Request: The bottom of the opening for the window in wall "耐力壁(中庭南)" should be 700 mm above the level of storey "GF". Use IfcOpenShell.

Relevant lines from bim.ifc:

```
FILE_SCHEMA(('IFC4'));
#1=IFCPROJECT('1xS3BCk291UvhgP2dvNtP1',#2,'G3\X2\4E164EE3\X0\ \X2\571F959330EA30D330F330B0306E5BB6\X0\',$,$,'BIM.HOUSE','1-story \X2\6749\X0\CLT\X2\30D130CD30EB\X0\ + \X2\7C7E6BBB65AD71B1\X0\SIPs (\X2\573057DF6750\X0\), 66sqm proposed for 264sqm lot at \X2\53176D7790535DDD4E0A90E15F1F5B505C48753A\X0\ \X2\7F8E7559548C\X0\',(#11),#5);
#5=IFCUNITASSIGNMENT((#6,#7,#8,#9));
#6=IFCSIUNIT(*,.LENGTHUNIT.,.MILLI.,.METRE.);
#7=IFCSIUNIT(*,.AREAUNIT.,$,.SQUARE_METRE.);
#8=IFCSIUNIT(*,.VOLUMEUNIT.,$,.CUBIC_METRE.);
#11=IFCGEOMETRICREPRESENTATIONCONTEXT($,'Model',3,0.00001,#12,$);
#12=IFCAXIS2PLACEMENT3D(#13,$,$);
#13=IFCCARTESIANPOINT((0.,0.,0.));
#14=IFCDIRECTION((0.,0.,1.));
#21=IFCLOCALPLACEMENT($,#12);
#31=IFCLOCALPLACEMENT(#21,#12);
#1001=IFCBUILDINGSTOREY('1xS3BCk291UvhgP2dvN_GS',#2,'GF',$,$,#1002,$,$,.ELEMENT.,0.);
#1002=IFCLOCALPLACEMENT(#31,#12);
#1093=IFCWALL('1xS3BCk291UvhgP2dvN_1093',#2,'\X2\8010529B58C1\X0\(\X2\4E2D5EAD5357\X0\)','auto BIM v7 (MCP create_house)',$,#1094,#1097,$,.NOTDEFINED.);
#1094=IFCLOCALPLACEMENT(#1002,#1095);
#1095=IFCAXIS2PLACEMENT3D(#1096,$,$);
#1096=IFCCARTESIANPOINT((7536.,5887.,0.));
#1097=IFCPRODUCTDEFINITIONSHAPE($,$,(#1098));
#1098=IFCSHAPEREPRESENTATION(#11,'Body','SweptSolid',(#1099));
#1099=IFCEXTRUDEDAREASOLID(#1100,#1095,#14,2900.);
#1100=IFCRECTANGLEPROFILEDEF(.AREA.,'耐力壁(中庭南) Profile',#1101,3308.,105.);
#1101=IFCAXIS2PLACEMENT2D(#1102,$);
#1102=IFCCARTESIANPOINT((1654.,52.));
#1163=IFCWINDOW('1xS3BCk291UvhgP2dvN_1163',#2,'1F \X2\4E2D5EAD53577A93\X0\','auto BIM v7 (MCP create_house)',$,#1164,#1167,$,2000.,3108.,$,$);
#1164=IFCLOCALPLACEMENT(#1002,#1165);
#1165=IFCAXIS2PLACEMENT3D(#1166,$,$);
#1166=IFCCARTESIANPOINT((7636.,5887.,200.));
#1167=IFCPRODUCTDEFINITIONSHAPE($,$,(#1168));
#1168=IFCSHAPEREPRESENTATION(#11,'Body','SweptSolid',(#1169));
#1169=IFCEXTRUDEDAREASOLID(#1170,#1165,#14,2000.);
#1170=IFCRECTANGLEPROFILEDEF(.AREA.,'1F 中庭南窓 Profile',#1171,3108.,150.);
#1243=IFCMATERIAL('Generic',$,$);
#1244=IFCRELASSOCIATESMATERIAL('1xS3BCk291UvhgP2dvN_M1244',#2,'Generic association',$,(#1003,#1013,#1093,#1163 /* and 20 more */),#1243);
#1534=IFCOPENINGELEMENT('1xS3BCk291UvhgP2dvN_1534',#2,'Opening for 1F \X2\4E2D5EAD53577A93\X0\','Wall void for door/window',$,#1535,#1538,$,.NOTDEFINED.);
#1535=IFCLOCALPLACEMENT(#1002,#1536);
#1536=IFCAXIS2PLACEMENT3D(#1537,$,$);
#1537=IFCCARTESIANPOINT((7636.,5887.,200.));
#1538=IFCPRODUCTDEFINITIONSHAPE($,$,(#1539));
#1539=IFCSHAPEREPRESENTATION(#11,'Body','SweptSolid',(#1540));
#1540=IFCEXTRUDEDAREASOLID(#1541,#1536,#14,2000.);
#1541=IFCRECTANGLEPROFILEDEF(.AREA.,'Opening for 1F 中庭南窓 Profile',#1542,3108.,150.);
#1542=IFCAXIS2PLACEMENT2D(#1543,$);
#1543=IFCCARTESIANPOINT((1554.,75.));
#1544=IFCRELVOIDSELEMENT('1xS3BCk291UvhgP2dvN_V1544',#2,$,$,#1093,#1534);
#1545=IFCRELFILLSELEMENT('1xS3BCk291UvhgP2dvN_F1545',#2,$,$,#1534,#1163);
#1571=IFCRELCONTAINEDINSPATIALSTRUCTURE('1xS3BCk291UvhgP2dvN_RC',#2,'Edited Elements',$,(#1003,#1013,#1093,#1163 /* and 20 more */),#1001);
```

```python
import numpy as np
import ifcopenshell
import ifcopenshell.api.geometry
import ifcopenshell.geom
import ifcopenshell.util.element
import ifcopenshell.util.placement
import ifcopenshell.util.shape
import ifcopenshell.util.unit

model = ifcopenshell.open("bim.ifc")
unit_scale = ifcopenshell.util.unit.calculate_unit_scale(model)

window = model.by_id(1163)
opening = window.FillsVoids[0].RelatingOpeningElement
storey = ifcopenshell.util.element.get_container(window, ifc_class="IfcBuildingStorey")
level = ifcopenshell.util.placement.get_local_placement(storey.ObjectPlacement)[2, 3]

# The opening's origin need not be at the sill, so measure its lowest point.
shape = ifcopenshell.geom.create_shape(ifcopenshell.geom.settings(), opening)
bottom = ifcopenshell.util.shape.get_shape_bottom_elevation(shape, shape.geometry) / unit_scale
dz = level + 700.0 - bottom

shift = np.array([0.0, 0.0, dz])
# The window is not placed relative to its opening, so move both.
for product in (opening, window):
    matrix = ifcopenshell.util.placement.get_local_placement(product.ObjectPlacement)
    matrix[:3, 3] += shift
    ifcopenshell.api.geometry.edit_object_placement(model, product=product, matrix=matrix, is_si=False)

print(f"moved by {dz * unit_scale:+.3f} m")

model.write("bim_edited.ifc")
```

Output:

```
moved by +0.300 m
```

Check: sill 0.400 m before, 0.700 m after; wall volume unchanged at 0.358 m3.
